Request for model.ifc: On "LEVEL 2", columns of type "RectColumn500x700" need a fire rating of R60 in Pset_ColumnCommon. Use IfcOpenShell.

First a look at what the model holds.

```python
import ifcopenshell
import ifcopenshell.util.element

model = ifcopenshell.open("model.ifc")
print(model.schema)
storey = next(s for s in model.by_type("IfcBuildingStorey") if s.Name == "LEVEL 2")
columns = [e for e in ifcopenshell.util.element.get_decomposition(storey) if e.is_a("IfcColumn")]
seen = {}
for e in columns:
    element_type = ifcopenshell.util.element.get_type(e)
    key = (element_type.Name if element_type != e and element_type else None, ifcopenshell.util.element.get_pset(e, "Pset_ColumnCommon", "FireRating"))
    seen[key] = seen.get(key, 0) + 1
for (name, value), count in sorted(seen.items(), key=str):
    print(count, "x", name, "|", value)
```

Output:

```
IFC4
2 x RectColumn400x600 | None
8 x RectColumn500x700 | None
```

```python
import ifcopenshell
import ifcopenshell.api.pset
import ifcopenshell.util.element

model = ifcopenshell.open("model.ifc")

storey = next(s for s in model.by_type("IfcBuildingStorey") if s.Name == "LEVEL 2")
columns = [e for e in ifcopenshell.util.element.get_decomposition(storey) if e.is_a("IfcColumn")]

count = 0
for e in columns:
    element_type = ifcopenshell.util.element.get_type(e)
    if element_type in (None, e) or element_type.Name != "RectColumn500x700":
        continue
    # add_pset returns the element's existing set when there is one.
    pset = ifcopenshell.api.pset.add_pset(model, product=e, name="Pset_ColumnCommon")
    ifcopenshell.api.pset.edit_pset(model, pset=pset, properties={"FireRating": "R60"})
    count += 1

print(count, "columns updated")

model.write("model_v2.ifc")
```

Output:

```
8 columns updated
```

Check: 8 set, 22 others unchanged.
